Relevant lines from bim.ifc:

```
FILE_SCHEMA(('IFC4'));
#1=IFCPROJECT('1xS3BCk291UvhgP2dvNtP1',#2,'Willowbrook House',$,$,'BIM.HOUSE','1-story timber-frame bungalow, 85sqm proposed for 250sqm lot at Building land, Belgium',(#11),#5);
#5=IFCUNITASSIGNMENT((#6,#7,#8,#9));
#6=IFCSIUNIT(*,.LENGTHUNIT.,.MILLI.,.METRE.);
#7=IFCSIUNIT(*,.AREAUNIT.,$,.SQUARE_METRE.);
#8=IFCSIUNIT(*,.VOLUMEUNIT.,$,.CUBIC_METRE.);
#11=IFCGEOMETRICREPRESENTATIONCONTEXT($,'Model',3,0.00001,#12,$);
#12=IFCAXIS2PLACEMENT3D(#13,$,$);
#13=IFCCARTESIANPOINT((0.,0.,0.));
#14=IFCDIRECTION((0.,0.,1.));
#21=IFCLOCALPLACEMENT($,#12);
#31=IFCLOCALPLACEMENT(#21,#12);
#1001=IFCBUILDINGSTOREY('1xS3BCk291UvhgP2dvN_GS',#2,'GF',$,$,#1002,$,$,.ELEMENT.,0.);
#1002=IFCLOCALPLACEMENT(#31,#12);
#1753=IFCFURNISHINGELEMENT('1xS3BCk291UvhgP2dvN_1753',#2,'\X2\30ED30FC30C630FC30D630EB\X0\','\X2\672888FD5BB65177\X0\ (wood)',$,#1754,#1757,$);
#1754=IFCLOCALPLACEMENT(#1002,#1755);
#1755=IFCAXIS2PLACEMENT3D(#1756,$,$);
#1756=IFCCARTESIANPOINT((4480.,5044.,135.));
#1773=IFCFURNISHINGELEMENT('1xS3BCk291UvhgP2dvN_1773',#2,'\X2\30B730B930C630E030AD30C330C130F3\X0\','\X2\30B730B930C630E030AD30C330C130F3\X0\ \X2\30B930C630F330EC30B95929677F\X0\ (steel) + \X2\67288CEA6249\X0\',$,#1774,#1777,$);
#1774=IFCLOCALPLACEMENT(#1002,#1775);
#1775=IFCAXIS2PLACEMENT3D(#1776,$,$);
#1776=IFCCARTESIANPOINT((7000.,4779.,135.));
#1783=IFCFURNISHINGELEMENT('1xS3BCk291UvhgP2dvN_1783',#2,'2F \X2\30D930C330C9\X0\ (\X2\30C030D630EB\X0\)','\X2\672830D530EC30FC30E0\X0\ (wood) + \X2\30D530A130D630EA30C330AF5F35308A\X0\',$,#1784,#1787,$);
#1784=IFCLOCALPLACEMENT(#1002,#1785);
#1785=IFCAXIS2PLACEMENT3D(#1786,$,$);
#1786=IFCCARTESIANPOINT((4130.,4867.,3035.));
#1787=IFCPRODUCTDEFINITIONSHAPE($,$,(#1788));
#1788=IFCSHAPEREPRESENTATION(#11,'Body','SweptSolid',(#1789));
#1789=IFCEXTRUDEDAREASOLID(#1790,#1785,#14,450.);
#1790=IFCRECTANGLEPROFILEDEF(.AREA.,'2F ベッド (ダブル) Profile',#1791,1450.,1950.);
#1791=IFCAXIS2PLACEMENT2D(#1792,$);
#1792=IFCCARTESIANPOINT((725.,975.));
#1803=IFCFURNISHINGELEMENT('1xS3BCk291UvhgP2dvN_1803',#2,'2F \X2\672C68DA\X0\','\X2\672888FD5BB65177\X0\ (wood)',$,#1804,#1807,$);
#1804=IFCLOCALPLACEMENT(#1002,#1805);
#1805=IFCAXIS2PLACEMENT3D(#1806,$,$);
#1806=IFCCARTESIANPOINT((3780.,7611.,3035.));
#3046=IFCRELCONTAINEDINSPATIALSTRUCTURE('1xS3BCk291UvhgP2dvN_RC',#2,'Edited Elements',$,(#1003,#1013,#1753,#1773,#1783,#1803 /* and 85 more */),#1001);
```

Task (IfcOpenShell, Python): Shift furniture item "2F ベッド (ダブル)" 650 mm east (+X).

```python
import ifcopenshell
import ifcopenshell.api.geometry
import ifcopenshell.util.placement

model = ifcopenshell.open("bim.ifc")

item = model.by_guid("1xS3BCk291UvhgP2dvN_1783")
matrix = ifcopenshell.util.placement.get_local_placement(item.ObjectPlacement)
matrix[0, 3] += 650.0
ifcopenshell.api.geometry.edit_object_placement(model, product=item, matrix=matrix, is_si=False)

print(ifcopenshell.util.placement.get_local_placement(item.ObjectPlacement).round(3) + 0.0)

model.write("bim_updated.ifc")
```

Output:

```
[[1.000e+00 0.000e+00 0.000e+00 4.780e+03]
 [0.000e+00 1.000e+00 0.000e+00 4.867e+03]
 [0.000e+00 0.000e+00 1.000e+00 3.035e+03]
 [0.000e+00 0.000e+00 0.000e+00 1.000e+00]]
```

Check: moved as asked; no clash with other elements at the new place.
